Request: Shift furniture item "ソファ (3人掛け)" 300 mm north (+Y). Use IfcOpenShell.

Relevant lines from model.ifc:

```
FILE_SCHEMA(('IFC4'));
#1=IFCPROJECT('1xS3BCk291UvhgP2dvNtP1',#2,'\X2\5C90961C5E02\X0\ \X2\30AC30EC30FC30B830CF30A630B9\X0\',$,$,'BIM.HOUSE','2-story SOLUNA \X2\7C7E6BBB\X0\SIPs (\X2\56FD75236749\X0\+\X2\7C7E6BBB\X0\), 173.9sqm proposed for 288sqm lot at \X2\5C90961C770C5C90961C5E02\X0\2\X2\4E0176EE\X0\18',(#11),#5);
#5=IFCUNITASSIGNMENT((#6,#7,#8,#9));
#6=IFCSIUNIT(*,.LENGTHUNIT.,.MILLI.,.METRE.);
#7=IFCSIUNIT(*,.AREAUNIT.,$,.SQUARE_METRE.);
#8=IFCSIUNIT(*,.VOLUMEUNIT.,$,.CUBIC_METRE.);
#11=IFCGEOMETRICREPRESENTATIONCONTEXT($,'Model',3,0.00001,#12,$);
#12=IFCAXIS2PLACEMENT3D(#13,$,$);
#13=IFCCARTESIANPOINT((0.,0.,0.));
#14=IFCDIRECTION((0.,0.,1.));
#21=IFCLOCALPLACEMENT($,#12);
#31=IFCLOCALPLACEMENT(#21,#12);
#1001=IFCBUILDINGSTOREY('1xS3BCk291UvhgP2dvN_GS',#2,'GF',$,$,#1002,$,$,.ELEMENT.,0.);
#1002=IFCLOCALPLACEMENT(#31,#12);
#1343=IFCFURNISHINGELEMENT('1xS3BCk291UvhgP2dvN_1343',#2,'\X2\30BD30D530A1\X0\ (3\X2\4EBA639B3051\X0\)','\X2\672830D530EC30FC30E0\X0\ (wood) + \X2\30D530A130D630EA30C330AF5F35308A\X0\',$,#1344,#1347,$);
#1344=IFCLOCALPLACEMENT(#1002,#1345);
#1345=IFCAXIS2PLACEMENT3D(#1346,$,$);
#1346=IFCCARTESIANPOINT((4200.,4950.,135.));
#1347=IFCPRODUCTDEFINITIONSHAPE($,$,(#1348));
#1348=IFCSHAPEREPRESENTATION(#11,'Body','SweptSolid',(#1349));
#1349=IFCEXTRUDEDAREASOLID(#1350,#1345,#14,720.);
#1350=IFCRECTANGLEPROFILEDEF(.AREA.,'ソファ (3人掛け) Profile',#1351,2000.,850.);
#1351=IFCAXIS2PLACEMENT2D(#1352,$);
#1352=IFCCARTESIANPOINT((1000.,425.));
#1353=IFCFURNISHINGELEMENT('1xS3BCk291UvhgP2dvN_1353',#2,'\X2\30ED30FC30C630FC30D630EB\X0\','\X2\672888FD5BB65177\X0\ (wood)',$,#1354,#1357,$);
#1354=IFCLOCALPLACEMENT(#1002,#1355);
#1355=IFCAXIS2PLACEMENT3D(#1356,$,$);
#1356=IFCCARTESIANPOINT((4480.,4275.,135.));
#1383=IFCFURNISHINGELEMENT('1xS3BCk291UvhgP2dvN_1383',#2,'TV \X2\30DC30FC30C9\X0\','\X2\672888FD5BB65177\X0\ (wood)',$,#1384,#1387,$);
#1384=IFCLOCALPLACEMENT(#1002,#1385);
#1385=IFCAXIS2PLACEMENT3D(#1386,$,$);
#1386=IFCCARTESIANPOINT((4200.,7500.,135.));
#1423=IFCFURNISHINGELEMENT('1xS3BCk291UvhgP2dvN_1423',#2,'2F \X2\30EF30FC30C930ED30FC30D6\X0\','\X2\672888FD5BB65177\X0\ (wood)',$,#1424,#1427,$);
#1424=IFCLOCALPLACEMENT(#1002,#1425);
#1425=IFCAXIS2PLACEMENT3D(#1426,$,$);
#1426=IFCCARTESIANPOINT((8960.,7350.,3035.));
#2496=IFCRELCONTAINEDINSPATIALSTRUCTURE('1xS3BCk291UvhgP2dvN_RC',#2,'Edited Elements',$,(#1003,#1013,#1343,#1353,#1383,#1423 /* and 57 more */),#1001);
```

```python
import ifcopenshell
import ifcopenshell.api.geometry
import ifcopenshell.util.placement
import ifcopenshell.util.unit

model = ifcopenshell.open("model.ifc")
unit_scale = ifcopenshell.util.unit.calculate_unit_scale(model)

item = model.by_guid("1xS3BCk291UvhgP2dvN_1343")
matrix = ifcopenshell.util.placement.get_local_placement(item.ObjectPlacement)
matrix[1, 3] += 0.3 / unit_scale
ifcopenshell.api.geometry.edit_object_placement(model, product=item, matrix=matrix, is_si=False)

print(ifcopenshell.util.placement.get_local_placement(item.ObjectPlacement).round(3) + 0.0)

model.write("model_edited.ifc")
```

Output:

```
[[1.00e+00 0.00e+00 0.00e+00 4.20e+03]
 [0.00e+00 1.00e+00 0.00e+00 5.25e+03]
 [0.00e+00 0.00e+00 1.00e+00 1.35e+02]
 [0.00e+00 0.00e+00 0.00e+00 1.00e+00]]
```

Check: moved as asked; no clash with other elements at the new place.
